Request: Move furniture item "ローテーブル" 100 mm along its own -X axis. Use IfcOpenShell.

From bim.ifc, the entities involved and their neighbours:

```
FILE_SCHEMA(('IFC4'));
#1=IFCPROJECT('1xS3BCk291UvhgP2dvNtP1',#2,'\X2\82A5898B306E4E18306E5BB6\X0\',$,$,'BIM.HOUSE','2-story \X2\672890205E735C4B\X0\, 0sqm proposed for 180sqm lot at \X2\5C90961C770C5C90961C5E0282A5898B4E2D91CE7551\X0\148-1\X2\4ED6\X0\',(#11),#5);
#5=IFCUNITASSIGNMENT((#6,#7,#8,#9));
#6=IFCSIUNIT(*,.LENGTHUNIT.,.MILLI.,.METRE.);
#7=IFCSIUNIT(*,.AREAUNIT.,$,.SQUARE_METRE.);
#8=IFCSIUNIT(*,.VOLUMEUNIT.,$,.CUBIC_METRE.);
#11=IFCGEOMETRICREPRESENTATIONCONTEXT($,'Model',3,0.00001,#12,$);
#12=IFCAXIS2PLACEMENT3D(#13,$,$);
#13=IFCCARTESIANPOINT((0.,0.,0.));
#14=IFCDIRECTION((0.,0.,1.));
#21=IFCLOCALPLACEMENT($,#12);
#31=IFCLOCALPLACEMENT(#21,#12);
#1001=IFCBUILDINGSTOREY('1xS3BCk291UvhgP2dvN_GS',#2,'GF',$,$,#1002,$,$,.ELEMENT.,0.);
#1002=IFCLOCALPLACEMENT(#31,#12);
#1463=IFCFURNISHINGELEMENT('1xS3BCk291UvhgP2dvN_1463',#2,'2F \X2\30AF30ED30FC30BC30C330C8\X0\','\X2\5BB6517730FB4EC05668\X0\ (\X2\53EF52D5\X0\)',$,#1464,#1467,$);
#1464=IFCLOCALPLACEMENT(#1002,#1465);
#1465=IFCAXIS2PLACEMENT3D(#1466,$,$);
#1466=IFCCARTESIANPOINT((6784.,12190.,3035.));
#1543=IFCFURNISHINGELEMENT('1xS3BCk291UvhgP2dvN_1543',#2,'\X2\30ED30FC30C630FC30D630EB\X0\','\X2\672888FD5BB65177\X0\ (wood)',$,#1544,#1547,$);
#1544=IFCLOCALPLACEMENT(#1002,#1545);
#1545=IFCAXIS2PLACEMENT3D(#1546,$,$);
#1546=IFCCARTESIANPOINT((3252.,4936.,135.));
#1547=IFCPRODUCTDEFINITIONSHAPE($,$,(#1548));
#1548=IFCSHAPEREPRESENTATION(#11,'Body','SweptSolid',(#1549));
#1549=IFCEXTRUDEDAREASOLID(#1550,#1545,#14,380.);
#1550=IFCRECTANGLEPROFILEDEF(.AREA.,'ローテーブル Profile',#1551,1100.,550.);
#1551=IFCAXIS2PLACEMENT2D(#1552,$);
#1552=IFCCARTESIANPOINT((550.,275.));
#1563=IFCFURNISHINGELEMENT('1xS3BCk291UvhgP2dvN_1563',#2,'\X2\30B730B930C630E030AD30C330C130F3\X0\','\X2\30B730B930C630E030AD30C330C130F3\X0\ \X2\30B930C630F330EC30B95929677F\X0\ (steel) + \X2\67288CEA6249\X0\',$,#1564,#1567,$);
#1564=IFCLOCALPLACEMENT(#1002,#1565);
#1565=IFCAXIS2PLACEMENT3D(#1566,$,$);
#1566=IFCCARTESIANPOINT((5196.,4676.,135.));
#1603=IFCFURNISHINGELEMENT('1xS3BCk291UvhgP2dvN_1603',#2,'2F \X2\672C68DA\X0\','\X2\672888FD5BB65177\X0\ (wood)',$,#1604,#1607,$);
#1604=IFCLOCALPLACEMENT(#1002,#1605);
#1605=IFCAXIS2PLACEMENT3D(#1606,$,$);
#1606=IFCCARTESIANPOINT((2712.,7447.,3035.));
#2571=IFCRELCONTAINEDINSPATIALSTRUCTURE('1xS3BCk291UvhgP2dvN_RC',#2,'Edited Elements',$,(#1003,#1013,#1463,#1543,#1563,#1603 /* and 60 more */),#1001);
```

```python
import ifcopenshell
import ifcopenshell.api.geometry
import ifcopenshell.util.placement

model = ifcopenshell.open("bim.ifc")

item = model.by_guid("1xS3BCk291UvhgP2dvN_1543")
matrix = ifcopenshell.util.placement.get_local_placement(item.ObjectPlacement)
matrix[:3, 3] -= matrix[:3, 0] * 100.0
ifcopenshell.api.geometry.edit_object_placement(model, product=item, matrix=matrix, is_si=False)

print(ifcopenshell.util.placement.get_local_placement(item.ObjectPlacement).round(3) + 0.0)

model.write("bim-out.ifc")
```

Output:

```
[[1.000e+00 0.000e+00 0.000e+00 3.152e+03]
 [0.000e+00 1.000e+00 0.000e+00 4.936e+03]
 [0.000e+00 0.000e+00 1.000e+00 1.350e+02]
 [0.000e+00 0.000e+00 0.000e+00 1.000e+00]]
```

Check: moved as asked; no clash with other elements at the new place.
